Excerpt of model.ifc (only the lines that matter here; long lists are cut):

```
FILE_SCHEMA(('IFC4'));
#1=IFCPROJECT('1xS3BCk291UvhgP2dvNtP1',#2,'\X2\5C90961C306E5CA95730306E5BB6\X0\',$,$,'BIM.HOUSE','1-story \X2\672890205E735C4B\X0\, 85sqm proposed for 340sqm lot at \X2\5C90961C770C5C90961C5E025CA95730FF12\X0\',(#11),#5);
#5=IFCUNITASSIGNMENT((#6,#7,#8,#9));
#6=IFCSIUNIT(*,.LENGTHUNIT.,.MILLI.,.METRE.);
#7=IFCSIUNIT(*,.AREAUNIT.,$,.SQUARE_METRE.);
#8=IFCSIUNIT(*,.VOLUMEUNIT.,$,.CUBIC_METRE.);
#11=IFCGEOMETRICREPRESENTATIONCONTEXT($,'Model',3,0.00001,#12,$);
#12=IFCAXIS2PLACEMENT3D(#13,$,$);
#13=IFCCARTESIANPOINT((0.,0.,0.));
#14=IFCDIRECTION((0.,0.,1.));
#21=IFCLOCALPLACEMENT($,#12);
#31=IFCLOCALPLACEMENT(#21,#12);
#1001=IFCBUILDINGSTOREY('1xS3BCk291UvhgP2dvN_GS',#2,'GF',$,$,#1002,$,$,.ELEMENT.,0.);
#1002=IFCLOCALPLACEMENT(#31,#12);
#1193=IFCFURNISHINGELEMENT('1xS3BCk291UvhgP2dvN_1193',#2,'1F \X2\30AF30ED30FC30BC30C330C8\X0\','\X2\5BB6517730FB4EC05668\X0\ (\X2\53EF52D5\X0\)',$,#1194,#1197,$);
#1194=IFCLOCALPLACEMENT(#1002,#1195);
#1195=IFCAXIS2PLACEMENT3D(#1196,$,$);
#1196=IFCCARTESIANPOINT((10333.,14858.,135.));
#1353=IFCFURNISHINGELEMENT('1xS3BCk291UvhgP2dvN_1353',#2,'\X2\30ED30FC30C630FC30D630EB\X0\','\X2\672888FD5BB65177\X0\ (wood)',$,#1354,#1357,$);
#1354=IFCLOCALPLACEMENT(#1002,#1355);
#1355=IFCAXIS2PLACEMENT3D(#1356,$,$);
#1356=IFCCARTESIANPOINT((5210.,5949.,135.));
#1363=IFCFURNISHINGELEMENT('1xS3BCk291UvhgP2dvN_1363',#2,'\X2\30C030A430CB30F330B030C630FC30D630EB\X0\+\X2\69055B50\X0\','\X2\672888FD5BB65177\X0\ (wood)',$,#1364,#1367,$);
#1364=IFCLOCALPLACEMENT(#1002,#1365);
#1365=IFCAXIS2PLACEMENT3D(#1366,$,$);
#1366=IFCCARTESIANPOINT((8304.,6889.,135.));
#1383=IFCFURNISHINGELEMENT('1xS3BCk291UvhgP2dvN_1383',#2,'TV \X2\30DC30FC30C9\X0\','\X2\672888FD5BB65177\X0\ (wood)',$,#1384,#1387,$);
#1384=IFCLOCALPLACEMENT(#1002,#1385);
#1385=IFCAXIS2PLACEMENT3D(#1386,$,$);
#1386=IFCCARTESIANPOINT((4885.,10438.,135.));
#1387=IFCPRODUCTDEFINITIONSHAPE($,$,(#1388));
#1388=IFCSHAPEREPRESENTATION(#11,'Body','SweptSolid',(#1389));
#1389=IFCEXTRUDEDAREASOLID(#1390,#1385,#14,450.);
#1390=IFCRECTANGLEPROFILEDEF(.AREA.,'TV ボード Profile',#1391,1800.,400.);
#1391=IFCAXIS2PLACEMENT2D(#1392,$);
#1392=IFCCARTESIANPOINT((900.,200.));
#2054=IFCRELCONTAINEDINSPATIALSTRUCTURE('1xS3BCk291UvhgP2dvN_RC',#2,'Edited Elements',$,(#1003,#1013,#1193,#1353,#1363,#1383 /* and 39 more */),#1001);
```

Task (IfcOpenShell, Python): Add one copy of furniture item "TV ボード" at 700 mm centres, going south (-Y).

```python
import numpy as np
import ifcopenshell
import ifcopenshell.api.geometry
import ifcopenshell.api.root
import ifcopenshell.util.element
import ifcopenshell.util.placement
import ifcopenshell.util.unit

model = ifcopenshell.open("model.ifc")
unit_scale = ifcopenshell.util.unit.calculate_unit_scale(model)


def reuse_history(source, copy):
    """copy_class also copies each property set's owner history, people and application; keep the originals."""
    for rel in copy.IsDefinedBy:
        if rel.is_a("IfcRelDefinesByProperties") and (history := rel.RelatingPropertyDefinition.OwnerHistory):
            rel.RelatingPropertyDefinition.OwnerHistory = source.OwnerHistory
            ifcopenshell.util.element.remove_deep2(model, history)


source = model.by_guid("1xS3BCk291UvhgP2dvN_1383")
base = ifcopenshell.util.placement.get_local_placement(source.ObjectPlacement)
step = np.array([0.0, -1.0, 0.0]) * 0.7 / unit_scale

for i in range(1, 2):
    copy = ifcopenshell.api.root.copy_class(model, product=source)
    copy.Representation = ifcopenshell.util.element.copy_deep(
        model, source.Representation, exclude=["IfcGeometricRepresentationContext", "IfcRepresentationMap"]
    )
    reuse_history(source, copy)
    matrix = base.copy()
    matrix[:3, 3] += i * step
    print("added at", matrix[:3, 3].round(3) + 0.0)
    ifcopenshell.api.geometry.edit_object_placement(model, product=copy, matrix=matrix, is_si=False)

model.write("model_v2.ifc")
```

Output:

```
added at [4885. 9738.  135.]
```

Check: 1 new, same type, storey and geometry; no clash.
